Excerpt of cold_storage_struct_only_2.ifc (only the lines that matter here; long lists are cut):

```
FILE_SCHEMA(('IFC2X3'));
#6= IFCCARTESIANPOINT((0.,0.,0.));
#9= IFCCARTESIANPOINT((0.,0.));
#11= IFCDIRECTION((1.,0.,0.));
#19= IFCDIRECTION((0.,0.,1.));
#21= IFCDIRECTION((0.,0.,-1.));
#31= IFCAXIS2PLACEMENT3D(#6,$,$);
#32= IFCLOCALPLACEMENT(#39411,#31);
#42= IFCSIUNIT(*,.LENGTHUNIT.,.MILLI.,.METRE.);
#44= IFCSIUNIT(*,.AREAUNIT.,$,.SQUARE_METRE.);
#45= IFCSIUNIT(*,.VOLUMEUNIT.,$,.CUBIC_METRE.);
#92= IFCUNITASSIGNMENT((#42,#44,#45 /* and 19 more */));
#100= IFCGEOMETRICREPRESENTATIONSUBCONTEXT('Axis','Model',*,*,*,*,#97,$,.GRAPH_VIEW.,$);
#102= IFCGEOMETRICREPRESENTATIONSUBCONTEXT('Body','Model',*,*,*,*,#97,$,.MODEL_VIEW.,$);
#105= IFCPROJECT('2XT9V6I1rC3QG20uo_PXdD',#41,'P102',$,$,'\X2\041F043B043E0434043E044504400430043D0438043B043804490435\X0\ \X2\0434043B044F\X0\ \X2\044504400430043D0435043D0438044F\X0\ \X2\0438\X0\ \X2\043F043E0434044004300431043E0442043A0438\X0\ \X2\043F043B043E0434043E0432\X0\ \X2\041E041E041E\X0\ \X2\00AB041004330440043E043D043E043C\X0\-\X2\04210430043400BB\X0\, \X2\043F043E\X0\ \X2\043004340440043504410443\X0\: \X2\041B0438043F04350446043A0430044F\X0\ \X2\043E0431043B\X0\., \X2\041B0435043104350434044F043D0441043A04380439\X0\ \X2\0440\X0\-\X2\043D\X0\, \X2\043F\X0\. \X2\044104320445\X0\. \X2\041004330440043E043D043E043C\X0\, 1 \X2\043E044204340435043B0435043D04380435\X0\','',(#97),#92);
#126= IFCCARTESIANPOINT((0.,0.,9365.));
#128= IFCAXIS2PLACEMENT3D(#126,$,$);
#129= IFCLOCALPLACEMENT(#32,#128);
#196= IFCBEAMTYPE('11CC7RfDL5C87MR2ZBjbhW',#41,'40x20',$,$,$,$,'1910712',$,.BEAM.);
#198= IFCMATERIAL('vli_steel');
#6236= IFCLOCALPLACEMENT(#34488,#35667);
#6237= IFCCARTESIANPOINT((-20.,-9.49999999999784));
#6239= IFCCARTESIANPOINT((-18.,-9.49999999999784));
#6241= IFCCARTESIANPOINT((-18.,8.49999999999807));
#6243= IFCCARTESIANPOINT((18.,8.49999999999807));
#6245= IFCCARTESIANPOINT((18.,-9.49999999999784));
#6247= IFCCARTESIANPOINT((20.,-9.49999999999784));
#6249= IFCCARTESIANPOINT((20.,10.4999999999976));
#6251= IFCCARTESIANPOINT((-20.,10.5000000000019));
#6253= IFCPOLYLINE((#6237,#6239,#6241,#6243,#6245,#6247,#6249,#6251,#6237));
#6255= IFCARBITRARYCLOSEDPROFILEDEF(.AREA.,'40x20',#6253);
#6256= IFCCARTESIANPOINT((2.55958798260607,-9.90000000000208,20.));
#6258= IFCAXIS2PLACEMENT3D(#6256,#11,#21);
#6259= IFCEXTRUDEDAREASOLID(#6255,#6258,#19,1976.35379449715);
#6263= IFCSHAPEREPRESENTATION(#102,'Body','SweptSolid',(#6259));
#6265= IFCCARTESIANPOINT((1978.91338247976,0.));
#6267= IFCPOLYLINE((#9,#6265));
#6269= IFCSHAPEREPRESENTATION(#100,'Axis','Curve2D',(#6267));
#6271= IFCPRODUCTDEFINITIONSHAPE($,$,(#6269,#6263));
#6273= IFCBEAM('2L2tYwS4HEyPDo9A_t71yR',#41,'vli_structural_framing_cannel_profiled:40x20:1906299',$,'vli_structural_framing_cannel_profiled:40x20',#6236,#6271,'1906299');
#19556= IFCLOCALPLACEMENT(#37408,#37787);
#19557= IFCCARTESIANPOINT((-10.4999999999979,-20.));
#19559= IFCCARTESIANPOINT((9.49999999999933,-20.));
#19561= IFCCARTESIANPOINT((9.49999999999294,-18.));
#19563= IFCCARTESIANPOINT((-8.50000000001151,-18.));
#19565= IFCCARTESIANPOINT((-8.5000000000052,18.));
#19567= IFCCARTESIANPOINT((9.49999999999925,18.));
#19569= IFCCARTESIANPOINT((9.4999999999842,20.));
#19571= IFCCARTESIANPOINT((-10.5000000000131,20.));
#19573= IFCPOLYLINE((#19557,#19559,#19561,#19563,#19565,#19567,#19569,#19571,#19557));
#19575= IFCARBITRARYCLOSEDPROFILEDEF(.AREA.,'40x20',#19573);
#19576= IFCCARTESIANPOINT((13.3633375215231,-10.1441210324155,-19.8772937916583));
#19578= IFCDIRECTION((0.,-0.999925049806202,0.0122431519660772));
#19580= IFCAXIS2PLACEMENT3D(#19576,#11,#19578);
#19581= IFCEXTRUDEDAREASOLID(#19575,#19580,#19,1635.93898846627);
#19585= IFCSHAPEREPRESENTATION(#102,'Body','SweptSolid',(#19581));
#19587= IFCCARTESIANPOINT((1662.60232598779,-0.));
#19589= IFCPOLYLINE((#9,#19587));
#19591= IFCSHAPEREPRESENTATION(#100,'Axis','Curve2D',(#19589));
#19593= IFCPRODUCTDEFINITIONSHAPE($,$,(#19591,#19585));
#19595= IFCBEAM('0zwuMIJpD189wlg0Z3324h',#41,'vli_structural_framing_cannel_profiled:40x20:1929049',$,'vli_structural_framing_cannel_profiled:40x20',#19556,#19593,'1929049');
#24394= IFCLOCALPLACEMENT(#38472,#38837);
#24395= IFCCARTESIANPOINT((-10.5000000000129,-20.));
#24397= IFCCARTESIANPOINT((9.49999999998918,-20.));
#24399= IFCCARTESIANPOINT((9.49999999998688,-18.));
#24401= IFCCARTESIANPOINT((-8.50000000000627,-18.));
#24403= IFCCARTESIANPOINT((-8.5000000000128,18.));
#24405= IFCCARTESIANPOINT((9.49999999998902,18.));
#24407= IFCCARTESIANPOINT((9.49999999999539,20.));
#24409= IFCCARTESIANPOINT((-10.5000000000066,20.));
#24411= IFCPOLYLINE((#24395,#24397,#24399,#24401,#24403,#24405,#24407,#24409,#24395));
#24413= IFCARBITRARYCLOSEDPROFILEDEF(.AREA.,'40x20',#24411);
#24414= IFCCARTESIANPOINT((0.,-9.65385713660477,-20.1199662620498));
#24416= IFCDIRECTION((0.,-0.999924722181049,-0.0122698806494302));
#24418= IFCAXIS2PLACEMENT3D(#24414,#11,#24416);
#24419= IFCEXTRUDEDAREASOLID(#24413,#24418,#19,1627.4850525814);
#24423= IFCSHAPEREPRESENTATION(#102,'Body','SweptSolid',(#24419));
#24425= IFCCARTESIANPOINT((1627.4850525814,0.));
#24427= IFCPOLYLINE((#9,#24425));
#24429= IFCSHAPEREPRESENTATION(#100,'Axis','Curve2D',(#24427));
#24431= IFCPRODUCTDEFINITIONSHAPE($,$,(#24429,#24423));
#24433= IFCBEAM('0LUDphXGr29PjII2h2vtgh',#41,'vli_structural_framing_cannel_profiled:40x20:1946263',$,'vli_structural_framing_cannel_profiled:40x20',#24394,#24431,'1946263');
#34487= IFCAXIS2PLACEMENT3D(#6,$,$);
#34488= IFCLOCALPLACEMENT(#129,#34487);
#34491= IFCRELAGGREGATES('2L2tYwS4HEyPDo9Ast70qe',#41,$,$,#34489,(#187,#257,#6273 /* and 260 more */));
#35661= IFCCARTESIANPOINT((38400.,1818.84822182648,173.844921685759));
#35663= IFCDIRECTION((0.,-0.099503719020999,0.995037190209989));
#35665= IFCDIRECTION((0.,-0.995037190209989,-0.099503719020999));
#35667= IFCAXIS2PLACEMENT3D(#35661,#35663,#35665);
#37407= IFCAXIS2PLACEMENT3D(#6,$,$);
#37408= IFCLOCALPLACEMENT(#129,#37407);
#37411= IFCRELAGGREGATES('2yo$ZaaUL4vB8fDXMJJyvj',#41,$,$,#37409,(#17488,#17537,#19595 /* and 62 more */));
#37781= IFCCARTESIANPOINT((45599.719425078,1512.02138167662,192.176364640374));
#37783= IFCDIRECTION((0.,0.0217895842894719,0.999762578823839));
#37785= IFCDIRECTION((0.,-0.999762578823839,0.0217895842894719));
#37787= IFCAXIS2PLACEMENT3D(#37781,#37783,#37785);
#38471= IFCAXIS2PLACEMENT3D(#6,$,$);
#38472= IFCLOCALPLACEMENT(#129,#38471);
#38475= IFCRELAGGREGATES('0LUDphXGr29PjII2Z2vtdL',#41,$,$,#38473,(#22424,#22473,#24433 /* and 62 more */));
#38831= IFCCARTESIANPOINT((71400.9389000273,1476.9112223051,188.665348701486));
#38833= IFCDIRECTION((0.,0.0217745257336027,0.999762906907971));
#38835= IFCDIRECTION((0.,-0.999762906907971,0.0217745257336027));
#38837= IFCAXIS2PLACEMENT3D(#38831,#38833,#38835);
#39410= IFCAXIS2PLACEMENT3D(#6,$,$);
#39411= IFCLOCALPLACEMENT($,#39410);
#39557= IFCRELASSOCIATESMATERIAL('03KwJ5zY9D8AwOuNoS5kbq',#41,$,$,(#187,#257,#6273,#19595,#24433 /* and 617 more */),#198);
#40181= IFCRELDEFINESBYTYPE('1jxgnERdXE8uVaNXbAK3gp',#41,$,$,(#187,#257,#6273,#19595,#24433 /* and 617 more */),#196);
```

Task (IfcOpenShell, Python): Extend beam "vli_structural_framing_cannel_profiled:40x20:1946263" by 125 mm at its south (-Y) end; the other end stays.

```python
import numpy as np
import ifcopenshell
import ifcopenshell.util.representation
import ifcopenshell.util.unit

model = ifcopenshell.open("cold_storage_struct_only_2.ifc")
unit_scale = ifcopenshell.util.unit.calculate_unit_scale(model)

member = model.by_guid("0LUDphXGr29PjII2h2vtgh")
change = 0.125 / unit_scale

# The extrusion runs towards the end named, so only its depth changes.
body = ifcopenshell.util.representation.get_representation(member, "Model", "Body")
solid = body.Items[0]
old_length = solid.Depth
solid.Depth += change

# Move the axis end point with it.
axis = next(r for r in member.Representation.Representations if r.RepresentationIdentifier == "Axis").Items[0]
start, end = (np.array(p.Coordinates) for p in axis.Points)
end = end + (end - start) / np.linalg.norm(end - start) * change
point = model.createIfcCartesianPoint(end.tolist())
axis.Points = [axis.Points[0], point]

print(f"length {old_length:g} -> {solid.Depth:g}")

model.write("cold_storage_struct_only_2_edited.ifc")
```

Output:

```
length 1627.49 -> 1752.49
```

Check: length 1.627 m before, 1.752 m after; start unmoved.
